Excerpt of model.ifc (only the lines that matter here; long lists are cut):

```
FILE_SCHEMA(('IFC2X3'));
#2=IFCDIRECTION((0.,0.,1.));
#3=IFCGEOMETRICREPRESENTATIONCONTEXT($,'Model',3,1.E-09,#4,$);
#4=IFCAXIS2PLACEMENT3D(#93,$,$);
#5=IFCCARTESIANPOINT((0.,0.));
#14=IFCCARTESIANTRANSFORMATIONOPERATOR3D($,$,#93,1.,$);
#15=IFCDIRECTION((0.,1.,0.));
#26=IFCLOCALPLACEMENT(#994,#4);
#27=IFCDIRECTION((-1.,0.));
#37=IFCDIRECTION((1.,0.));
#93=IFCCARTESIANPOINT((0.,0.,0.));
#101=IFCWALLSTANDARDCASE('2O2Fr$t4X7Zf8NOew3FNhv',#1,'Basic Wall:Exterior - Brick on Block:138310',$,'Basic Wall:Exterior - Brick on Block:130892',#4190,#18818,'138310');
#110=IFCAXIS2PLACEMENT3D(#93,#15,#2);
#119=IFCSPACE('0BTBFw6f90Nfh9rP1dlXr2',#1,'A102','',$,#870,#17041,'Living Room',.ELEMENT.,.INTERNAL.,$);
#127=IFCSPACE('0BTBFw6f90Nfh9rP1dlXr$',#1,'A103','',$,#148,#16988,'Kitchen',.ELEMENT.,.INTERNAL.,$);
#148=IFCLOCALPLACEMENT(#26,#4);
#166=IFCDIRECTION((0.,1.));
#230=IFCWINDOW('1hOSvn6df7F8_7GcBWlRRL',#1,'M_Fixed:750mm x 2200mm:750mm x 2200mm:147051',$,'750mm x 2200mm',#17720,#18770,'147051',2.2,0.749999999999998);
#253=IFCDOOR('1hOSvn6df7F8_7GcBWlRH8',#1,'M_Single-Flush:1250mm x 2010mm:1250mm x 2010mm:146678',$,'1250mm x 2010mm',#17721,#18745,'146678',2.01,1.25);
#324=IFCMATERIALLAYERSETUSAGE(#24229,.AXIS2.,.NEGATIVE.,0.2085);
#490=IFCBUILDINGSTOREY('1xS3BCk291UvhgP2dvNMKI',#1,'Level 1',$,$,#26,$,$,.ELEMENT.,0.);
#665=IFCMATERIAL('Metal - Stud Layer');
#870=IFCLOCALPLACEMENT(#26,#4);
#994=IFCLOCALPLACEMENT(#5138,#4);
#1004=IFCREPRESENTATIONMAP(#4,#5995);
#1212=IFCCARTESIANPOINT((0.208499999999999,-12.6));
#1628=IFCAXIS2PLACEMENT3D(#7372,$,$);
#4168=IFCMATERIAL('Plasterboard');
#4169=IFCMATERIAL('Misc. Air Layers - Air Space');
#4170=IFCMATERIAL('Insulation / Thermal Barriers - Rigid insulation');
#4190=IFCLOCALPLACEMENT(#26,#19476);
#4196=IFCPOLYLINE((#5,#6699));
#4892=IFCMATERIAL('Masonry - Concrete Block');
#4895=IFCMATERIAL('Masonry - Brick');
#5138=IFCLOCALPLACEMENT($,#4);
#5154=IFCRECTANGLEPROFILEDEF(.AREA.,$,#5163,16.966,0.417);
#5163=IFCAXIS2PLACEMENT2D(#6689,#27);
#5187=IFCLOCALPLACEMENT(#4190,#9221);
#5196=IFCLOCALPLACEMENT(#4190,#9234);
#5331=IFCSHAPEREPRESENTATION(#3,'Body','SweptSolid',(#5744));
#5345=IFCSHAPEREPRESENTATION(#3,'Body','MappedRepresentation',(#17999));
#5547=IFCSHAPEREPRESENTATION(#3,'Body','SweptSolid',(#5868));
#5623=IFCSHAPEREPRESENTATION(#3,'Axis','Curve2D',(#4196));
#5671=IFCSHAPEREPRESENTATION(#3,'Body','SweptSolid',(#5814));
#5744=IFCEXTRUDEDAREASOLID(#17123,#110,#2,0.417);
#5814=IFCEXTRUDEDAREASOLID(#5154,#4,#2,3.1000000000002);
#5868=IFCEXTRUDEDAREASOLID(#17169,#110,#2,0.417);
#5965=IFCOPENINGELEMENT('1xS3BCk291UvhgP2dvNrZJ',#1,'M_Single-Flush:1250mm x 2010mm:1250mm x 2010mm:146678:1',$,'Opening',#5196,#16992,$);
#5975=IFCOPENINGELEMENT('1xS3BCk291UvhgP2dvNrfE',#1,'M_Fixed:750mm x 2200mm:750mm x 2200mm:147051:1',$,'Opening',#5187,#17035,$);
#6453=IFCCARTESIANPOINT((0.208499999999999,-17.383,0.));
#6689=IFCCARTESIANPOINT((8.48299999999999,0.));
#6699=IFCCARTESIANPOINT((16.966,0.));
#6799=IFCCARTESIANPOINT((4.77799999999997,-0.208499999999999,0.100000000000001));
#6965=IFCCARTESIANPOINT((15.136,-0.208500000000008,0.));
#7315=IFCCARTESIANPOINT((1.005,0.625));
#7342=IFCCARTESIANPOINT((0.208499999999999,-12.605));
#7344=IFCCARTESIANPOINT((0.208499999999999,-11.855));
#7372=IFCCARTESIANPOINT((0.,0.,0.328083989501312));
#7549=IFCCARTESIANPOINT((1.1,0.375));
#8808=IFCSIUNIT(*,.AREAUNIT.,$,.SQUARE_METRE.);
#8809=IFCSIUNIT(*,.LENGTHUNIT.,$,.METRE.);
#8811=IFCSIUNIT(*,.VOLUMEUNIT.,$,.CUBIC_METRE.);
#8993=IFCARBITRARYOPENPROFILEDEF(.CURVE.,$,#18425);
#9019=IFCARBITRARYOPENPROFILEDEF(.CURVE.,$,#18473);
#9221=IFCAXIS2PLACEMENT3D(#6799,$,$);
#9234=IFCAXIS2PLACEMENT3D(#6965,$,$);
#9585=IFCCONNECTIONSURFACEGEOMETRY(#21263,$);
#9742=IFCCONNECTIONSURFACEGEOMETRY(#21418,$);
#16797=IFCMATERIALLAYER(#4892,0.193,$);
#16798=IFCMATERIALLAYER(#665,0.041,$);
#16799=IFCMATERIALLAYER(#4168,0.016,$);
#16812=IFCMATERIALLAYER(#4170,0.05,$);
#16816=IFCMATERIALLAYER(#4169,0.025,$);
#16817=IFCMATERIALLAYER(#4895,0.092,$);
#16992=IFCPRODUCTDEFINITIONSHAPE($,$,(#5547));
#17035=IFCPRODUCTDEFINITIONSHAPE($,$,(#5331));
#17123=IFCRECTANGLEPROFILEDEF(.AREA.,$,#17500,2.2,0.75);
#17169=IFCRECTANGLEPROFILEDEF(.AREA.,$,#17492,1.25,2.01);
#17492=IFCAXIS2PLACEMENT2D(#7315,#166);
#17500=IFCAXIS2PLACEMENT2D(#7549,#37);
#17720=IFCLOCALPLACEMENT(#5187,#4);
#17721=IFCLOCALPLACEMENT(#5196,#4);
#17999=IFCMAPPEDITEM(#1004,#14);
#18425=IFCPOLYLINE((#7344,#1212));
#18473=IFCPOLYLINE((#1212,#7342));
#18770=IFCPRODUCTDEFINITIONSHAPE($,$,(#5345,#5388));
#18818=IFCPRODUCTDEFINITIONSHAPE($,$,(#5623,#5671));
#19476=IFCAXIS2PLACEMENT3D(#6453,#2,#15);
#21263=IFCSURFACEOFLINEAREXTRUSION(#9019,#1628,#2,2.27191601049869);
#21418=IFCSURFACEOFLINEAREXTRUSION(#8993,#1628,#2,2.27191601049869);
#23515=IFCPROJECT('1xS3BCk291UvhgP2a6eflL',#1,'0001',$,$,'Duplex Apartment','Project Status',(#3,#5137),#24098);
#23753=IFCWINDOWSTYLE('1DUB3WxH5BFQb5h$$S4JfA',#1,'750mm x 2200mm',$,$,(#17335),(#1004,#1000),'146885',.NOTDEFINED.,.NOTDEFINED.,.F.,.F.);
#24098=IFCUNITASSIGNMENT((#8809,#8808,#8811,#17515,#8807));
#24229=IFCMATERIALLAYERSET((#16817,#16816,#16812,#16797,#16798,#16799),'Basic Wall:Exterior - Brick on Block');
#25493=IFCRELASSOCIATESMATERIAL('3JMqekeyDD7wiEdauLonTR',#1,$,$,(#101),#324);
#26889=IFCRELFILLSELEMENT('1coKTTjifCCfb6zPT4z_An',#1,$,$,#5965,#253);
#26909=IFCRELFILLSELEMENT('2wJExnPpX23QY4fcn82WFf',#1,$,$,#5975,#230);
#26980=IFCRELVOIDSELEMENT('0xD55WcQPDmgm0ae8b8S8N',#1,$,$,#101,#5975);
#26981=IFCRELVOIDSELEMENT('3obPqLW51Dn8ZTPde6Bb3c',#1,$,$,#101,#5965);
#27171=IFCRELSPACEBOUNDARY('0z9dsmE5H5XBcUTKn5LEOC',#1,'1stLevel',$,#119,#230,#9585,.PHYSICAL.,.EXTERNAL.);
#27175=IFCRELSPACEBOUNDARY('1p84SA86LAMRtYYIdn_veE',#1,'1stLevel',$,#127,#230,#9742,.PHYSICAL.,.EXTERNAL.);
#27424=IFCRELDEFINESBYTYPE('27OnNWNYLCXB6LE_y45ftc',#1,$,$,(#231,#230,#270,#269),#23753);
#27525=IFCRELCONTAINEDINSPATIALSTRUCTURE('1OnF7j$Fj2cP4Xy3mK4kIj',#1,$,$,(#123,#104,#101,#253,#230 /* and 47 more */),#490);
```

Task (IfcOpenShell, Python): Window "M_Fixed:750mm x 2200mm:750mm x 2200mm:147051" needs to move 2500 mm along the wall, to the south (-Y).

```python
import numpy as np
import ifcopenshell
import ifcopenshell.api.geometry
import ifcopenshell.util.placement
import ifcopenshell.util.unit

model = ifcopenshell.open("model.ifc")
unit_scale = ifcopenshell.util.unit.calculate_unit_scale(model)

window = model.by_guid("1hOSvn6df7F8_7GcBWlRRL")
opening = window.FillsVoids[0].RelatingOpeningElement
wall = opening.VoidsElements[0].RelatingBuildingElement

wall_matrix = ifcopenshell.util.placement.get_local_placement(wall.ObjectPlacement)
shift = wall_matrix[:3, 0] * -2.5 / unit_scale
before = ifcopenshell.util.placement.get_local_placement(window.ObjectPlacement)[:3, 3].copy()

# The window is placed relative to its opening, so it follows when the opening moves.
matrix = ifcopenshell.util.placement.get_local_placement(opening.ObjectPlacement)
matrix[:3, 3] += shift
ifcopenshell.api.geometry.edit_object_placement(
    model, product=opening, matrix=matrix, is_si=False, should_transform_children=True
)

# Space boundary surfaces are stored in each space's coordinates; move them too.
for rel in window.ProvidesBoundaries:
    if not rel.ConnectionGeometry:
        continue
    surface = rel.ConnectionGeometry.SurfaceOnRelatingElement
    space_matrix = ifcopenshell.util.placement.get_local_placement(rel.RelatingSpace.ObjectPlacement)
    point = np.array(surface.Position.Location.Coordinates) + space_matrix[:3, :3].T @ shift
    surface.Position = model.createIfcAxis2Placement3D(
        model.createIfcCartesianPoint(point.tolist()), surface.Position.Axis, surface.Position.RefDirection
    )

after = ifcopenshell.util.placement.get_local_placement(window.ObjectPlacement)[:3, 3]
print("window moved by", (after - before).round(3) + 0.0)

model.write("model_rev.ifc")
```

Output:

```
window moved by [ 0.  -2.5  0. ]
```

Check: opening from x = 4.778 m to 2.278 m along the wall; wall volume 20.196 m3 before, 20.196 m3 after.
